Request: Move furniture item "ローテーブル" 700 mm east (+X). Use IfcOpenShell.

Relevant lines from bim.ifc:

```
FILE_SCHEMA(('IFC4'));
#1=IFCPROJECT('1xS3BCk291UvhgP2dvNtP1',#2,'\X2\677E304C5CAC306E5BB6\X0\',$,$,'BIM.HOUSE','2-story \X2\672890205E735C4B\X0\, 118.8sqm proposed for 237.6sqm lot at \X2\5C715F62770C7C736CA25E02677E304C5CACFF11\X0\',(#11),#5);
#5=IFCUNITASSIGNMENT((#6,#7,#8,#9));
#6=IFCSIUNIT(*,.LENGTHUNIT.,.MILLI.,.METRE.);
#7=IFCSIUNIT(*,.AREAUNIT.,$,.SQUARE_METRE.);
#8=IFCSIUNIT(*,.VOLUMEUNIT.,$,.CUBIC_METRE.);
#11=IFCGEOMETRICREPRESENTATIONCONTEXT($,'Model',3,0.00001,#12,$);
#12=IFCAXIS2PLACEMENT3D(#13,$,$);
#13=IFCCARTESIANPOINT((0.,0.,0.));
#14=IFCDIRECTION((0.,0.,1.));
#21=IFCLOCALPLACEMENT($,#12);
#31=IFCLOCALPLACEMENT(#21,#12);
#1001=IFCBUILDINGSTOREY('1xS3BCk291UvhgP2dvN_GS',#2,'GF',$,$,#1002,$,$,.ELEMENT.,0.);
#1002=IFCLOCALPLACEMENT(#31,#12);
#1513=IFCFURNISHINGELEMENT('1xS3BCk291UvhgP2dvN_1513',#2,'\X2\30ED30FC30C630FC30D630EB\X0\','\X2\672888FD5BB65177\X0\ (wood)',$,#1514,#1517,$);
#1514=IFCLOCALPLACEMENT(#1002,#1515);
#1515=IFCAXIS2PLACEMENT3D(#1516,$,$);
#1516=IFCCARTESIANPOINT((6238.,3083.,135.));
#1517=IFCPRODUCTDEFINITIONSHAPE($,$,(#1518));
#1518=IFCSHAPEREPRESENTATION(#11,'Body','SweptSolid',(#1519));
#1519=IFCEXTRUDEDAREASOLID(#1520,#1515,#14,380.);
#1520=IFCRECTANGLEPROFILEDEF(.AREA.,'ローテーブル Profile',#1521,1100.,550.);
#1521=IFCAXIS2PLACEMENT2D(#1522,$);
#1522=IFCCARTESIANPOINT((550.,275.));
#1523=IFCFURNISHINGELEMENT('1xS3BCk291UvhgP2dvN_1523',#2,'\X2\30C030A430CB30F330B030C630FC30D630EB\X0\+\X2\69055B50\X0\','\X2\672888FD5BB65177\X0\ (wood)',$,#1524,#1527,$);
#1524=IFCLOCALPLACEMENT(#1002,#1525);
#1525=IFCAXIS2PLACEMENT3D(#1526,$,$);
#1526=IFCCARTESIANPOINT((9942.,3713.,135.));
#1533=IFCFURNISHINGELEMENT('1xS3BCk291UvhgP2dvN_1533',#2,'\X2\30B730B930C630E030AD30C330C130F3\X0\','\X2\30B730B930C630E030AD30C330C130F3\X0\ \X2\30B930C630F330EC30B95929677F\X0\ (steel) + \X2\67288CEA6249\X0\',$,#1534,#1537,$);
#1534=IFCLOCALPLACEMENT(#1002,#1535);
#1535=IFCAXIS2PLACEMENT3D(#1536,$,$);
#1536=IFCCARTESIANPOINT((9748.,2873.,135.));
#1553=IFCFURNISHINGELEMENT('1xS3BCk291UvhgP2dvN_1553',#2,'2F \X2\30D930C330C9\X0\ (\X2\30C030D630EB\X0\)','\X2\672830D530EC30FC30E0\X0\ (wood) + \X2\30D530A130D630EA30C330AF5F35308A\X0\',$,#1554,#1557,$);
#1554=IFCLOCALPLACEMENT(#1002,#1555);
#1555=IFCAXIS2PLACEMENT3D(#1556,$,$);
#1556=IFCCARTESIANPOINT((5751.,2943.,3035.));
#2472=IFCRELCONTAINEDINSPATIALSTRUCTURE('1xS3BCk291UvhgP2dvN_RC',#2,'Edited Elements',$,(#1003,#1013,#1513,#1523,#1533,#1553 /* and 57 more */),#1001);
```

```python
import ifcopenshell
import ifcopenshell.api.geometry
import ifcopenshell.util.placement

model = ifcopenshell.open("bim.ifc")

item = model.by_guid("1xS3BCk291UvhgP2dvN_1513")
matrix = ifcopenshell.util.placement.get_local_placement(item.ObjectPlacement)
matrix[0, 3] += 700.0
ifcopenshell.api.geometry.edit_object_placement(model, product=item, matrix=matrix, is_si=False)

print(ifcopenshell.util.placement.get_local_placement(item.ObjectPlacement).round(3) + 0.0)

model.write("bim_rev.ifc")
```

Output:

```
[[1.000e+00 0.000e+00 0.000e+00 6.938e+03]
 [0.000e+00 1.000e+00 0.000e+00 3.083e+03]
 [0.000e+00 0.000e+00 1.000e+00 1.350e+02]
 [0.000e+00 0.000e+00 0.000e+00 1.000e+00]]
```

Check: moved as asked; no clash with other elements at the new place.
